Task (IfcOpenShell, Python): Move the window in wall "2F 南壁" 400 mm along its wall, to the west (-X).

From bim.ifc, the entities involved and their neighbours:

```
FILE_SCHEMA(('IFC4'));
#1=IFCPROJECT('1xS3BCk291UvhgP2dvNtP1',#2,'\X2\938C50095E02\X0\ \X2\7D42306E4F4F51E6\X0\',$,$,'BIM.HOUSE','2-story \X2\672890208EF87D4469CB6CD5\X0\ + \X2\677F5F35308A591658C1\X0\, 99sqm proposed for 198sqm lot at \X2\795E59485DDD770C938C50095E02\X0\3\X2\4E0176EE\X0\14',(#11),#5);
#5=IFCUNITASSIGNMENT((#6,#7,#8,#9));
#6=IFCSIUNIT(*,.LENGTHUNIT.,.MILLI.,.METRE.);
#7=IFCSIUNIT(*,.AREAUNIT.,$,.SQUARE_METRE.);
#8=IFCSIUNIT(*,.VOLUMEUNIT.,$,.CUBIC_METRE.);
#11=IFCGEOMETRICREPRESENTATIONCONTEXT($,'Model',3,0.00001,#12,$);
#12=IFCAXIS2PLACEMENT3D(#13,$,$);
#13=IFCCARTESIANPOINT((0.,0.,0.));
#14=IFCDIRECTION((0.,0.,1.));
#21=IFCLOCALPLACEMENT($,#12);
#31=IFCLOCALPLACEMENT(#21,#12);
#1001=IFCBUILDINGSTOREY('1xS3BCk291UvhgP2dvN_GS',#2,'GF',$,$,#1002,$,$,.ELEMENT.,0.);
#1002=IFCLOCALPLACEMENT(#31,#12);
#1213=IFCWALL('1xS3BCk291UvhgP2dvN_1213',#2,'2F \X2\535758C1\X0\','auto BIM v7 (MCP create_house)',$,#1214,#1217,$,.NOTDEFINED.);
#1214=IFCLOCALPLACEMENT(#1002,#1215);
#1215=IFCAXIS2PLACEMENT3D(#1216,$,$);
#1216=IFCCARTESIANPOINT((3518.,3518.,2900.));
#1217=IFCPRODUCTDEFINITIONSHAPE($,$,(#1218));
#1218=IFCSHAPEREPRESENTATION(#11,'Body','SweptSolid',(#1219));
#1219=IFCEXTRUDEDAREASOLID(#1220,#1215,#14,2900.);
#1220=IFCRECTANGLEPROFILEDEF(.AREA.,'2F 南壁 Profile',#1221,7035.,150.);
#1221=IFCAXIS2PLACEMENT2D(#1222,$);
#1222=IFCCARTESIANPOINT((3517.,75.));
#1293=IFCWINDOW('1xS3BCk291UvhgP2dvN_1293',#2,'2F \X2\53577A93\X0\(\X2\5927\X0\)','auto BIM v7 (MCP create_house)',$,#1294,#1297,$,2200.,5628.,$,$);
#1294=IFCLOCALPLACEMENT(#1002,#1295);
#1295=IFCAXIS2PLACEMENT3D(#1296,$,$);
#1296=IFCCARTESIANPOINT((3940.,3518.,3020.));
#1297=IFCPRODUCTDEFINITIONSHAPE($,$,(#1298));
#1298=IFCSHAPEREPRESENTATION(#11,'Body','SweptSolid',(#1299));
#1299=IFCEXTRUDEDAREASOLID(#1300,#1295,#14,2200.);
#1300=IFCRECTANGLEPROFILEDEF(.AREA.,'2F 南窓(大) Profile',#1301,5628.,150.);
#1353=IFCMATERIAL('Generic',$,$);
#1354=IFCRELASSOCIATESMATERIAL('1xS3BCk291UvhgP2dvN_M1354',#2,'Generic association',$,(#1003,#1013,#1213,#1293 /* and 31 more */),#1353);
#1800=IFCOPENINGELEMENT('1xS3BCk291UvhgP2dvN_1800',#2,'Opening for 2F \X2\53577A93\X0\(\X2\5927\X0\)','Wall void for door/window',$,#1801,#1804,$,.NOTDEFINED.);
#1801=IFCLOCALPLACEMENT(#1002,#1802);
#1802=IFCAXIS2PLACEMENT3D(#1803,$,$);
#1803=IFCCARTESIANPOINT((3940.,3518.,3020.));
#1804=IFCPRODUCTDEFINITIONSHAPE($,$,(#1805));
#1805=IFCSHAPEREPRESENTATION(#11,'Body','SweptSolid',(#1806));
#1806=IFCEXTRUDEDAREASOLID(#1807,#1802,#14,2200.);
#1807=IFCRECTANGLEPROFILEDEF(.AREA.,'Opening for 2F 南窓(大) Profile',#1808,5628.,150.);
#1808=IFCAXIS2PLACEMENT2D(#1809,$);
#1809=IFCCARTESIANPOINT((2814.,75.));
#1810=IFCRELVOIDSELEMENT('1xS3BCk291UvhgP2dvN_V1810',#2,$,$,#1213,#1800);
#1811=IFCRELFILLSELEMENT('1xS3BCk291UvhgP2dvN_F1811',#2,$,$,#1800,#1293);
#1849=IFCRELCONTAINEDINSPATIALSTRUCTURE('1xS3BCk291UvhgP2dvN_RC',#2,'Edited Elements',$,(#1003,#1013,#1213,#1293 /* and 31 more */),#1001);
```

```python
import ifcopenshell
import ifcopenshell.api.geometry
import ifcopenshell.util.placement

model = ifcopenshell.open("bim.ifc")

window = model.by_guid("1xS3BCk291UvhgP2dvN_1293")
opening = window.FillsVoids[0].RelatingOpeningElement
wall = opening.VoidsElements[0].RelatingBuildingElement

wall_matrix = ifcopenshell.util.placement.get_local_placement(wall.ObjectPlacement)
shift = wall_matrix[:3, 0] * -400.0
before = ifcopenshell.util.placement.get_local_placement(window.ObjectPlacement)[:3, 3].copy()

# The window is not placed relative to its opening, so move both.
for product in (opening, window):
    matrix = ifcopenshell.util.placement.get_local_placement(product.ObjectPlacement)
    matrix[:3, 3] += shift
    ifcopenshell.api.geometry.edit_object_placement(model, product=product, matrix=matrix, is_si=False)

after = ifcopenshell.util.placement.get_local_placement(window.ObjectPlacement)[:3, 3]
print("window moved by", (after - before).round(3) + 0.0)

model.write("bim_updated.ifc")
```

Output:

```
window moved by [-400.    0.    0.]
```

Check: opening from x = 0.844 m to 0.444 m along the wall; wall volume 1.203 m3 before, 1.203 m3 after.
